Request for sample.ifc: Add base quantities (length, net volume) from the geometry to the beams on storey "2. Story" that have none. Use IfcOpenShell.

First a look at what the model holds.

```python
import ifcopenshell
import ifcopenshell.util.element
import ifcopenshell.util.unit

model = ifcopenshell.open("sample.ifc")
print(model.schema)
for unit_type in ("LENGTHUNIT", "AREAUNIT", "VOLUMEUNIT"):
    print(unit_type, ifcopenshell.util.unit.calculate_unit_scale(model, unit_type))
storey = next(s for s in model.by_type("IfcBuildingStorey") if s.Name == "2. Story")
beams = [e for e in ifcopenshell.util.element.get_decomposition(storey) if e.is_a("IfcBeam")]
for e in sorted(beams, key=lambda e: e.id()):
    print(e.id(), e.is_a(), e.Name, list(ifcopenshell.util.element.get_psets(e, qtos_only=True)), sep=" | ")
```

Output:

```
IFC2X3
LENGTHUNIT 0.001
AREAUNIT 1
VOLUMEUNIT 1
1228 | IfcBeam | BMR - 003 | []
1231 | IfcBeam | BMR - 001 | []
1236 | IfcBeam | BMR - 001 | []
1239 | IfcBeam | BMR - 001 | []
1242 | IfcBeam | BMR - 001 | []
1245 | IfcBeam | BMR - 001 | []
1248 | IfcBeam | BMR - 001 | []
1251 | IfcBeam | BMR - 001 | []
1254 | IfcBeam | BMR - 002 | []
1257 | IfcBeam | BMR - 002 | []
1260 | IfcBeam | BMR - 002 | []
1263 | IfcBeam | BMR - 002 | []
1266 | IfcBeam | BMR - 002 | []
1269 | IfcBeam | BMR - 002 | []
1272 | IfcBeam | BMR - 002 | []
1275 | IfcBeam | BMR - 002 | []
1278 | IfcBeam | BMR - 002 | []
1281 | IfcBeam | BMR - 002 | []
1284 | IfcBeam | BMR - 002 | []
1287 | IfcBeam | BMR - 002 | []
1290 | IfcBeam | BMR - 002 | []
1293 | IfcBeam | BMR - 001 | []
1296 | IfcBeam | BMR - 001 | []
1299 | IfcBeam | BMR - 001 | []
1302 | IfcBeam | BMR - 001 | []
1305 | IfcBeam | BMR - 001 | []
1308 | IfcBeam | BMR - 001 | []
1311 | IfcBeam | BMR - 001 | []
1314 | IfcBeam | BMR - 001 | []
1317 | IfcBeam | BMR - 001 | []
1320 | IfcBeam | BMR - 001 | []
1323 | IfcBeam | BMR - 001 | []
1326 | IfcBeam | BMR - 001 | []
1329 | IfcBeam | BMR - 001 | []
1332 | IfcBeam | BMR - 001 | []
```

```python
import ifcopenshell
import ifcopenshell.api.pset
import ifcopenshell.geom
import ifcopenshell.util.element
import ifcopenshell.util.shape
import ifcopenshell.util.unit

model = ifcopenshell.open("sample.ifc")
unit_scale = ifcopenshell.util.unit.calculate_unit_scale(model)
volume_scale = ifcopenshell.util.unit.calculate_unit_scale(model, "VOLUMEUNIT")
settings = ifcopenshell.geom.settings()

storey = next(s for s in model.by_type("IfcBuildingStorey") if s.Name == "2. Story")
beams = [e for e in ifcopenshell.util.element.get_decomposition(storey) if e.is_a("IfcBeam")]

for e in sorted(beams, key=lambda e: e.id()):
    if ifcopenshell.util.element.get_psets(e, qtos_only=True, should_inherit=False):
        continue
    # Geometry comes back in metres, in the element's own axes.
    shape = ifcopenshell.geom.create_shape(settings, e)
    values = {
        "Length": ifcopenshell.util.shape.get_max_xyz(shape.geometry) / unit_scale,
        "NetVolume": ifcopenshell.util.shape.get_volume(shape.geometry) / volume_scale,
    }
    qto = ifcopenshell.api.pset.add_qto(model, product=e, name="BaseQuantities")
    ifcopenshell.api.pset.edit_qto(model, qto=qto, properties=values)
    print(e.id(), {k: round(v, 3) for k, v in values.items()})

model.write("sample_updated.ifc")
```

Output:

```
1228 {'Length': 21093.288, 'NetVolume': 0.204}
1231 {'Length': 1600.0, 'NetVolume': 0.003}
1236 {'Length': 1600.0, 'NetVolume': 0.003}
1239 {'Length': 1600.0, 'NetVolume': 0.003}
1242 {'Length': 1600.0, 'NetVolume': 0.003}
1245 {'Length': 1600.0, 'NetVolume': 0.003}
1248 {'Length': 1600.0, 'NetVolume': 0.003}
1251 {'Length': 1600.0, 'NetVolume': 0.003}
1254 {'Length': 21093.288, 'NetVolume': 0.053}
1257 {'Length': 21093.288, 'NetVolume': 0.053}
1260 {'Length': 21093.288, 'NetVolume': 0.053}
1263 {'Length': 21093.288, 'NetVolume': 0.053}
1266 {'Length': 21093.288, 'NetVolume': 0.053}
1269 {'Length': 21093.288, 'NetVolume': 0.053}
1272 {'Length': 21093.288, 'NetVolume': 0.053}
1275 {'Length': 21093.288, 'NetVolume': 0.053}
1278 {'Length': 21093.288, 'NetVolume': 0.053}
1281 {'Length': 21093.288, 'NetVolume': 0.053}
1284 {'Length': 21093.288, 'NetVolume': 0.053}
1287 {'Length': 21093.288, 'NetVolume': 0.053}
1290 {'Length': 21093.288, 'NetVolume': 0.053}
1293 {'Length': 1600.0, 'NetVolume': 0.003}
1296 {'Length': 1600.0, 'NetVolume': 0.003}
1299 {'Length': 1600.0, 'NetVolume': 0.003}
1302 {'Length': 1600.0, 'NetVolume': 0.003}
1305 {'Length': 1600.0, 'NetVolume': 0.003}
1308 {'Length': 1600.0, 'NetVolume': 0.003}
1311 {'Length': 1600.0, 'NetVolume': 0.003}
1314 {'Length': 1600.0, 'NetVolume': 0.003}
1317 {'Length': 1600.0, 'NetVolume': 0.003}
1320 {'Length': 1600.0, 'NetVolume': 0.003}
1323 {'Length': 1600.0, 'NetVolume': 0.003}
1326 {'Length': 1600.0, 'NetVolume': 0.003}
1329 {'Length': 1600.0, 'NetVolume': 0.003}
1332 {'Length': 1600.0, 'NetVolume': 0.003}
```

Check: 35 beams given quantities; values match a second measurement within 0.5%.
